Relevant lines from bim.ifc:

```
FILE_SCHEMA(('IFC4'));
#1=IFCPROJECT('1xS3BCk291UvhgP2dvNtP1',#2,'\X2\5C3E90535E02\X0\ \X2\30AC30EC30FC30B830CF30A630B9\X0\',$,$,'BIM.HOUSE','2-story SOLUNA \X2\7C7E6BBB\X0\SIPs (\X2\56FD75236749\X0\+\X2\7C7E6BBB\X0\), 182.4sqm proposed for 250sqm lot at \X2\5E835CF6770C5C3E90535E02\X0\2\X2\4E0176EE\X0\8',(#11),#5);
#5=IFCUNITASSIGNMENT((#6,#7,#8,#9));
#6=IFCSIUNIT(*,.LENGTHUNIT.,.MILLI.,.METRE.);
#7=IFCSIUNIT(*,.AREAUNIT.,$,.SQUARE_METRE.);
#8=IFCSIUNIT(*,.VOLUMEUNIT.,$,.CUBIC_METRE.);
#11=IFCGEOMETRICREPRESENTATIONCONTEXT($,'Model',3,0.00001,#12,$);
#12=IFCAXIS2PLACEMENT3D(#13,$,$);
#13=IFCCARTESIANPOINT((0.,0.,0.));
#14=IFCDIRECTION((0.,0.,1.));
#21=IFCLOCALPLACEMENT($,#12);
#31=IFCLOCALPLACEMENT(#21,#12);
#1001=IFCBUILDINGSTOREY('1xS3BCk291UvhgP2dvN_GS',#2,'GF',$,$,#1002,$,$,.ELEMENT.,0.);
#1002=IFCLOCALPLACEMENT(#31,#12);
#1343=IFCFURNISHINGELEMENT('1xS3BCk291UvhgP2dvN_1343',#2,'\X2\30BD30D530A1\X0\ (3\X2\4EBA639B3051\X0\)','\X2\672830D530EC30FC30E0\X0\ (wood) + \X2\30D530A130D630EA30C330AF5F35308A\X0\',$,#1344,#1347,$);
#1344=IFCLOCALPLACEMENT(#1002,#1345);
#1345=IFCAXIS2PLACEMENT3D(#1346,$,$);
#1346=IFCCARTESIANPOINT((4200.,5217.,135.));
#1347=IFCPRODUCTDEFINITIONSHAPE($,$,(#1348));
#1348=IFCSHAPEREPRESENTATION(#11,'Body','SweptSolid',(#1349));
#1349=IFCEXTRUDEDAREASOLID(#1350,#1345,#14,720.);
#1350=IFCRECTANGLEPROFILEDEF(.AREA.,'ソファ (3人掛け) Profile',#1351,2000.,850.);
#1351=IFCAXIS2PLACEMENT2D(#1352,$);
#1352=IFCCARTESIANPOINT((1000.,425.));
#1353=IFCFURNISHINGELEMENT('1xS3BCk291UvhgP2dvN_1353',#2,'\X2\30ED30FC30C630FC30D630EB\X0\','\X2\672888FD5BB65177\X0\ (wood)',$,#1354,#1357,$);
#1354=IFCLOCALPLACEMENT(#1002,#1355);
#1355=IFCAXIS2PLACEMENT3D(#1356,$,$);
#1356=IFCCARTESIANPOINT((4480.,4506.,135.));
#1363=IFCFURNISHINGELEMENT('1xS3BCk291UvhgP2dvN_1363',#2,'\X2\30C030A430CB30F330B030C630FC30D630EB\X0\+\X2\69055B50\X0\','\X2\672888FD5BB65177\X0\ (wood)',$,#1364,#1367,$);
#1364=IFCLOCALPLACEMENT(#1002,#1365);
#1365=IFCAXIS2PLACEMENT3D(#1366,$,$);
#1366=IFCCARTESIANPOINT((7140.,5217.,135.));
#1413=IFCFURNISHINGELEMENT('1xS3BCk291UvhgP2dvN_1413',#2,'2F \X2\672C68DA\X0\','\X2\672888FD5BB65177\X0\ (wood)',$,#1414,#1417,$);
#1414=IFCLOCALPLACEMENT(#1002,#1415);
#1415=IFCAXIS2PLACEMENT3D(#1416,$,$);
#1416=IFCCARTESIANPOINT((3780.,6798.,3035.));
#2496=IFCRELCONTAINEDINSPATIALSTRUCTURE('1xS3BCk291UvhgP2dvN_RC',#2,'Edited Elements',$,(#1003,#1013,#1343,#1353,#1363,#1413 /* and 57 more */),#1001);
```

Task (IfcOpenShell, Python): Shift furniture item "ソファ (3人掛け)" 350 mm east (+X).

```python
import ifcopenshell
import ifcopenshell.api.geometry
import ifcopenshell.util.placement

model = ifcopenshell.open("bim.ifc")

item = model.by_id(1343)
matrix = ifcopenshell.util.placement.get_local_placement(item.ObjectPlacement)
matrix[0, 3] += 350.0
ifcopenshell.api.geometry.edit_object_placement(model, product=item, matrix=matrix, is_si=False)

print(ifcopenshell.util.placement.get_local_placement(item.ObjectPlacement).round(3) + 0.0)

model.write("bim_updated.ifc")
```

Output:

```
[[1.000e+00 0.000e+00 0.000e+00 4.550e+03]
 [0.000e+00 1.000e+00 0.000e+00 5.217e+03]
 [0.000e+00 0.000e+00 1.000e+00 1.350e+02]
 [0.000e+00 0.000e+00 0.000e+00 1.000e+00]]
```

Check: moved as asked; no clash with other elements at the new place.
